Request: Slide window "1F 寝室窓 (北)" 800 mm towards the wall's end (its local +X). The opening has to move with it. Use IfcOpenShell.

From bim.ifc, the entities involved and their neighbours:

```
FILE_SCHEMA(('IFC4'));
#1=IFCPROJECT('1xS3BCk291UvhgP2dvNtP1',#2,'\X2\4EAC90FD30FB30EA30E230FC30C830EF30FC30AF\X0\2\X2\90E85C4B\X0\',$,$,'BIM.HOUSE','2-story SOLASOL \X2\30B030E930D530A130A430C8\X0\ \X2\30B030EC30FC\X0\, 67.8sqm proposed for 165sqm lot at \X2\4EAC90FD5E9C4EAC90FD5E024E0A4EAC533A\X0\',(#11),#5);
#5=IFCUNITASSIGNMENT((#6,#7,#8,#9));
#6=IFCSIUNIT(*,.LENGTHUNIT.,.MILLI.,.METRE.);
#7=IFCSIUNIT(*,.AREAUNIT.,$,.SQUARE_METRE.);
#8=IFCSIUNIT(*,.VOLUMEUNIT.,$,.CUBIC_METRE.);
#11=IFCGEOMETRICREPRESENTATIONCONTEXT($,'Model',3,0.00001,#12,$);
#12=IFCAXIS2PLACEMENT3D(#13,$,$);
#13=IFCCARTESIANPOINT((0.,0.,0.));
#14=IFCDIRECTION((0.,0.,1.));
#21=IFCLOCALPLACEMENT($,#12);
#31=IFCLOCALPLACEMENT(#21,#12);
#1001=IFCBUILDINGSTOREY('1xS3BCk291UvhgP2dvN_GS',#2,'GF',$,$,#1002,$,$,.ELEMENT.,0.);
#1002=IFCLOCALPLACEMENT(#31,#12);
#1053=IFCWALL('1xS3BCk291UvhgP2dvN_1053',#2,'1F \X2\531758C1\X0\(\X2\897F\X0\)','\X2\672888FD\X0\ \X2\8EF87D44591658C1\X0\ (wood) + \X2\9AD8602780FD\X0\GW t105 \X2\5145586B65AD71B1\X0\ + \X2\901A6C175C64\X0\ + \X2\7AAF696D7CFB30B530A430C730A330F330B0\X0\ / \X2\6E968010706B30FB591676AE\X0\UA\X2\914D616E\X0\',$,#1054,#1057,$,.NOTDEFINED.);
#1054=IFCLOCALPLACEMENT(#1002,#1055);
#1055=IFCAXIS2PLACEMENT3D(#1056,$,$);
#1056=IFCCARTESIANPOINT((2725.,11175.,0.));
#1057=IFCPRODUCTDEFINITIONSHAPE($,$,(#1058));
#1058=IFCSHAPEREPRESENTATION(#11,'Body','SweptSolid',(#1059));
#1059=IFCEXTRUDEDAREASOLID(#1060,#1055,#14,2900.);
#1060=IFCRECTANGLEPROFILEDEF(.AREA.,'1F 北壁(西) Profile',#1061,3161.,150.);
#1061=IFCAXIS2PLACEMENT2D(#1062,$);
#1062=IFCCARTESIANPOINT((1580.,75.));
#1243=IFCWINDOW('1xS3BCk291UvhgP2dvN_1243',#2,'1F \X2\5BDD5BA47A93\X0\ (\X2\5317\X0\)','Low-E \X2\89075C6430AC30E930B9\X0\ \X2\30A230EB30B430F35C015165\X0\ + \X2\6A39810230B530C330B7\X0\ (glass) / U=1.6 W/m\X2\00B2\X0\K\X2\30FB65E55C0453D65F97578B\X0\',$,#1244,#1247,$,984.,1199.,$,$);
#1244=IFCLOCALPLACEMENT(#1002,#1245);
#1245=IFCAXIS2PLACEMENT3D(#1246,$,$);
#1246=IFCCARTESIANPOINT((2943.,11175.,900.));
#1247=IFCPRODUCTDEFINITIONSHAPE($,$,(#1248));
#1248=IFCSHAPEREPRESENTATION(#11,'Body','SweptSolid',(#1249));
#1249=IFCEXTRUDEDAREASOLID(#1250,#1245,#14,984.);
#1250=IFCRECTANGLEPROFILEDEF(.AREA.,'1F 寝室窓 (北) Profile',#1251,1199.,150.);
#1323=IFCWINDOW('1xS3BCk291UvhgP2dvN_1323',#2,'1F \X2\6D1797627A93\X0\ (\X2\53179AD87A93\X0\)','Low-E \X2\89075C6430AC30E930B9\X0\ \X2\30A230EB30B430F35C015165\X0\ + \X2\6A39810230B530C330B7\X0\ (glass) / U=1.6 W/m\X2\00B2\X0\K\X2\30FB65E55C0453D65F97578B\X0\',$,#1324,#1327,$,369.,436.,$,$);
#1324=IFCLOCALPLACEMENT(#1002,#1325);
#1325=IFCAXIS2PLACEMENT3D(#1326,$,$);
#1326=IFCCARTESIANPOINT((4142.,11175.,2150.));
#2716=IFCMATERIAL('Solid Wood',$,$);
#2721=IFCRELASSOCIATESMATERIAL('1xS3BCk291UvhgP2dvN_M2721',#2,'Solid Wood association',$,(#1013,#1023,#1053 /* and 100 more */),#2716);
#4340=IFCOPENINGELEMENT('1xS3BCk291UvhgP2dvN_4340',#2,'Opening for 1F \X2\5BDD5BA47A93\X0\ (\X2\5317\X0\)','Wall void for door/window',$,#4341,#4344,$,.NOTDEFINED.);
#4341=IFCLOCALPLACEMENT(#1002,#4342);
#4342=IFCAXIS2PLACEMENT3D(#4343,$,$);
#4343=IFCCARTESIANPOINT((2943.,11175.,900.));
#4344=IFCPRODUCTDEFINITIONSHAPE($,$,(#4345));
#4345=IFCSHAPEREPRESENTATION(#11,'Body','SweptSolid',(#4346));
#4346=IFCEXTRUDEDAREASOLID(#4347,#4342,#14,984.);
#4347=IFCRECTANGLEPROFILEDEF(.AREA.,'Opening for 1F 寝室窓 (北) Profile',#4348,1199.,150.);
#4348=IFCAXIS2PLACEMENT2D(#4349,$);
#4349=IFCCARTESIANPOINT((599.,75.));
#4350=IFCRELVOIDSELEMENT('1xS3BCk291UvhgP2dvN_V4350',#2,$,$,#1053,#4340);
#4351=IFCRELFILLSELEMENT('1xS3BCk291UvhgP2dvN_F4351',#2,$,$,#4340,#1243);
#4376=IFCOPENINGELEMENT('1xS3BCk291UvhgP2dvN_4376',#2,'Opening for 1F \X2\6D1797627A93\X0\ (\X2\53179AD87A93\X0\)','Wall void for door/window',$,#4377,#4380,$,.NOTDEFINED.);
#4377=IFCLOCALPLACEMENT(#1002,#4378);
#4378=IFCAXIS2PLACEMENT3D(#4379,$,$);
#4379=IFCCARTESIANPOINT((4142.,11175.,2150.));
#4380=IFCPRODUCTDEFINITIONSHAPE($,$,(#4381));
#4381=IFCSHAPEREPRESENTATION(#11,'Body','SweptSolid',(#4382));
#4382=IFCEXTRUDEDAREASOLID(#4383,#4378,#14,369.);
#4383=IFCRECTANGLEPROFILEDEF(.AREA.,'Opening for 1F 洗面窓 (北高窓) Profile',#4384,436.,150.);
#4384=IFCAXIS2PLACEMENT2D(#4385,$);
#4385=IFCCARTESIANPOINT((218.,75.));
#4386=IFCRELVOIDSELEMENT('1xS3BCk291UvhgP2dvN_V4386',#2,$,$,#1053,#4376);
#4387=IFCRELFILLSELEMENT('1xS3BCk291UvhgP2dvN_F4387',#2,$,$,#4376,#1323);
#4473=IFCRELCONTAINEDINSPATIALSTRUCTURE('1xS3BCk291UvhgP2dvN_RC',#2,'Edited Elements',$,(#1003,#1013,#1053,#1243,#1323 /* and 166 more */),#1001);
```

```python
import ifcopenshell
import ifcopenshell.api.geometry
import ifcopenshell.util.placement
import ifcopenshell.util.unit

model = ifcopenshell.open("bim.ifc")
unit_scale = ifcopenshell.util.unit.calculate_unit_scale(model)

window = model.by_id(1243)
opening = window.FillsVoids[0].RelatingOpeningElement
wall = opening.VoidsElements[0].RelatingBuildingElement

wall_matrix = ifcopenshell.util.placement.get_local_placement(wall.ObjectPlacement)
shift = wall_matrix[:3, 0] * 0.8 / unit_scale
before = ifcopenshell.util.placement.get_local_placement(window.ObjectPlacement)[:3, 3].copy()

# The window is not placed relative to its opening, so move both.
for product in (opening, window):
    matrix = ifcopenshell.util.placement.get_local_placement(product.ObjectPlacement)
    matrix[:3, 3] += shift
    ifcopenshell.api.geometry.edit_object_placement(model, product=product, matrix=matrix, is_si=False)

after = ifcopenshell.util.placement.get_local_placement(window.ObjectPlacement)[:3, 3]
print("window moved by", (after - before).round(3) + 0.0)

model.write("bim_rev.ifc")
```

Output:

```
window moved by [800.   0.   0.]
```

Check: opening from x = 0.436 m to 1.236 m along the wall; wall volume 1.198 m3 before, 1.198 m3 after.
